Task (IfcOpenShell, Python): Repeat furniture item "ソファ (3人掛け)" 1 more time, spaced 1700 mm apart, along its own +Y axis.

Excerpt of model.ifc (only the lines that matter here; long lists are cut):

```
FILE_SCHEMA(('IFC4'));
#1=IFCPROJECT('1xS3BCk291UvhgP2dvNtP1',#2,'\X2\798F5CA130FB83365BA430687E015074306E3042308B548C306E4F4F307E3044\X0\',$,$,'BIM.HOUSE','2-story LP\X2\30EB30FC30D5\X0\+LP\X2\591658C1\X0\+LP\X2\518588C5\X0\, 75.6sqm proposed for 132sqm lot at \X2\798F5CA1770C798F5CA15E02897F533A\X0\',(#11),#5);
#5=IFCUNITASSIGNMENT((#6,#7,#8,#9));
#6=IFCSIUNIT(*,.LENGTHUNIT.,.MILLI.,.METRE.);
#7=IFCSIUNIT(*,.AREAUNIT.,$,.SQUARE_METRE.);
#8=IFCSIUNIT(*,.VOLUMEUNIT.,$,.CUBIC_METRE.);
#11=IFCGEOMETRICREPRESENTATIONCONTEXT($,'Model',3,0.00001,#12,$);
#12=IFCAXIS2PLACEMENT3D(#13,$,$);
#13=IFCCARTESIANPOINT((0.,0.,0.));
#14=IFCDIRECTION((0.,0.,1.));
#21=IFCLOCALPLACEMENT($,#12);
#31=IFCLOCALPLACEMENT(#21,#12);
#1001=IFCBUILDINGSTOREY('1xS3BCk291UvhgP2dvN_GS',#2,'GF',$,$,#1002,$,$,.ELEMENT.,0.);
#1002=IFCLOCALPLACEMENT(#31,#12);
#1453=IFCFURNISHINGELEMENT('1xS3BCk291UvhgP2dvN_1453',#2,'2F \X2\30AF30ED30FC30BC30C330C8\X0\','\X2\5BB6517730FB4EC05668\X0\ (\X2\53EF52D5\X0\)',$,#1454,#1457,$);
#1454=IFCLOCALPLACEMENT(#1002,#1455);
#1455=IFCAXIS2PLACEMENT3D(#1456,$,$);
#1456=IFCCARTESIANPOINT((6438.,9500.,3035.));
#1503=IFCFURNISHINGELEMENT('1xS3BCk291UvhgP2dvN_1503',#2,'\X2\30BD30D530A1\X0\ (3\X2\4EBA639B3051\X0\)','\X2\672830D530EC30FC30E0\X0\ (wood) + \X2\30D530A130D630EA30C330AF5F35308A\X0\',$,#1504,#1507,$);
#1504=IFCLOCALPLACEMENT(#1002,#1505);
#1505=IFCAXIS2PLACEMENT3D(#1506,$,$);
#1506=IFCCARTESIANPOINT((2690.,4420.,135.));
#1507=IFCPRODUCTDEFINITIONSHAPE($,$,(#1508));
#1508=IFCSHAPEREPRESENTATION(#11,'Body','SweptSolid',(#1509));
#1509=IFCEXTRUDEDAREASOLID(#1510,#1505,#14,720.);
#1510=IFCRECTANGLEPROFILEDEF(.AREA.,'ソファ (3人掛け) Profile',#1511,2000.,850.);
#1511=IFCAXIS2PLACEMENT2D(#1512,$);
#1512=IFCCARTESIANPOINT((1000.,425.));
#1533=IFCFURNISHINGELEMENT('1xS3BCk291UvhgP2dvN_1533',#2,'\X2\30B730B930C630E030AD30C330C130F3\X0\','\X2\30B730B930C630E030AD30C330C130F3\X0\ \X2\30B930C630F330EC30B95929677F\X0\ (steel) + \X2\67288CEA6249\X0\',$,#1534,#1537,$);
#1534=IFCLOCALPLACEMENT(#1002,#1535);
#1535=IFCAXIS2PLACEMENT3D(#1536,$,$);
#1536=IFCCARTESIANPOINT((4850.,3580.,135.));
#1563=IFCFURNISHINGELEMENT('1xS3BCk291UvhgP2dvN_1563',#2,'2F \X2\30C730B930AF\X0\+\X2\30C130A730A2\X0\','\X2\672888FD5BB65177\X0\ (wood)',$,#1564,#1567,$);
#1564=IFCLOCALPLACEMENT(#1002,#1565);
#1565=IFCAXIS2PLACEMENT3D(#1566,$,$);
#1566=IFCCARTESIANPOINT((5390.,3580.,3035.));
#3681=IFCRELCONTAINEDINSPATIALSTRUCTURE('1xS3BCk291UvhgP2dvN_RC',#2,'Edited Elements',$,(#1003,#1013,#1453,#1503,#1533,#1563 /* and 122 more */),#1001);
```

```python
import ifcopenshell
import ifcopenshell.api.geometry
import ifcopenshell.api.root
import ifcopenshell.util.element
import ifcopenshell.util.placement

model = ifcopenshell.open("model.ifc")


def reuse_history(source, copy):
    """copy_class also copies each property set's owner history, people and application; keep the originals."""
    for rel in copy.IsDefinedBy:
        if rel.is_a("IfcRelDefinesByProperties") and (history := rel.RelatingPropertyDefinition.OwnerHistory):
            rel.RelatingPropertyDefinition.OwnerHistory = source.OwnerHistory
            ifcopenshell.util.element.remove_deep2(model, history)


source = model.by_id(1503)
base = ifcopenshell.util.placement.get_local_placement(source.ObjectPlacement)
step = base[:3, 1] * 1700.0

for i in range(1, 2):
    copy = ifcopenshell.api.root.copy_class(model, product=source)
    copy.Representation = ifcopenshell.util.element.copy_deep(
        model, source.Representation, exclude=["IfcGeometricRepresentationContext", "IfcRepresentationMap"]
    )
    reuse_history(source, copy)
    matrix = base.copy()
    matrix[:3, 3] += i * step
    print("added at", matrix[:3, 3].round(3) + 0.0)
    ifcopenshell.api.geometry.edit_object_placement(model, product=copy, matrix=matrix, is_si=False)

model.write("model-out.ifc")
```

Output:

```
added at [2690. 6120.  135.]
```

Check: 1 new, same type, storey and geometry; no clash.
